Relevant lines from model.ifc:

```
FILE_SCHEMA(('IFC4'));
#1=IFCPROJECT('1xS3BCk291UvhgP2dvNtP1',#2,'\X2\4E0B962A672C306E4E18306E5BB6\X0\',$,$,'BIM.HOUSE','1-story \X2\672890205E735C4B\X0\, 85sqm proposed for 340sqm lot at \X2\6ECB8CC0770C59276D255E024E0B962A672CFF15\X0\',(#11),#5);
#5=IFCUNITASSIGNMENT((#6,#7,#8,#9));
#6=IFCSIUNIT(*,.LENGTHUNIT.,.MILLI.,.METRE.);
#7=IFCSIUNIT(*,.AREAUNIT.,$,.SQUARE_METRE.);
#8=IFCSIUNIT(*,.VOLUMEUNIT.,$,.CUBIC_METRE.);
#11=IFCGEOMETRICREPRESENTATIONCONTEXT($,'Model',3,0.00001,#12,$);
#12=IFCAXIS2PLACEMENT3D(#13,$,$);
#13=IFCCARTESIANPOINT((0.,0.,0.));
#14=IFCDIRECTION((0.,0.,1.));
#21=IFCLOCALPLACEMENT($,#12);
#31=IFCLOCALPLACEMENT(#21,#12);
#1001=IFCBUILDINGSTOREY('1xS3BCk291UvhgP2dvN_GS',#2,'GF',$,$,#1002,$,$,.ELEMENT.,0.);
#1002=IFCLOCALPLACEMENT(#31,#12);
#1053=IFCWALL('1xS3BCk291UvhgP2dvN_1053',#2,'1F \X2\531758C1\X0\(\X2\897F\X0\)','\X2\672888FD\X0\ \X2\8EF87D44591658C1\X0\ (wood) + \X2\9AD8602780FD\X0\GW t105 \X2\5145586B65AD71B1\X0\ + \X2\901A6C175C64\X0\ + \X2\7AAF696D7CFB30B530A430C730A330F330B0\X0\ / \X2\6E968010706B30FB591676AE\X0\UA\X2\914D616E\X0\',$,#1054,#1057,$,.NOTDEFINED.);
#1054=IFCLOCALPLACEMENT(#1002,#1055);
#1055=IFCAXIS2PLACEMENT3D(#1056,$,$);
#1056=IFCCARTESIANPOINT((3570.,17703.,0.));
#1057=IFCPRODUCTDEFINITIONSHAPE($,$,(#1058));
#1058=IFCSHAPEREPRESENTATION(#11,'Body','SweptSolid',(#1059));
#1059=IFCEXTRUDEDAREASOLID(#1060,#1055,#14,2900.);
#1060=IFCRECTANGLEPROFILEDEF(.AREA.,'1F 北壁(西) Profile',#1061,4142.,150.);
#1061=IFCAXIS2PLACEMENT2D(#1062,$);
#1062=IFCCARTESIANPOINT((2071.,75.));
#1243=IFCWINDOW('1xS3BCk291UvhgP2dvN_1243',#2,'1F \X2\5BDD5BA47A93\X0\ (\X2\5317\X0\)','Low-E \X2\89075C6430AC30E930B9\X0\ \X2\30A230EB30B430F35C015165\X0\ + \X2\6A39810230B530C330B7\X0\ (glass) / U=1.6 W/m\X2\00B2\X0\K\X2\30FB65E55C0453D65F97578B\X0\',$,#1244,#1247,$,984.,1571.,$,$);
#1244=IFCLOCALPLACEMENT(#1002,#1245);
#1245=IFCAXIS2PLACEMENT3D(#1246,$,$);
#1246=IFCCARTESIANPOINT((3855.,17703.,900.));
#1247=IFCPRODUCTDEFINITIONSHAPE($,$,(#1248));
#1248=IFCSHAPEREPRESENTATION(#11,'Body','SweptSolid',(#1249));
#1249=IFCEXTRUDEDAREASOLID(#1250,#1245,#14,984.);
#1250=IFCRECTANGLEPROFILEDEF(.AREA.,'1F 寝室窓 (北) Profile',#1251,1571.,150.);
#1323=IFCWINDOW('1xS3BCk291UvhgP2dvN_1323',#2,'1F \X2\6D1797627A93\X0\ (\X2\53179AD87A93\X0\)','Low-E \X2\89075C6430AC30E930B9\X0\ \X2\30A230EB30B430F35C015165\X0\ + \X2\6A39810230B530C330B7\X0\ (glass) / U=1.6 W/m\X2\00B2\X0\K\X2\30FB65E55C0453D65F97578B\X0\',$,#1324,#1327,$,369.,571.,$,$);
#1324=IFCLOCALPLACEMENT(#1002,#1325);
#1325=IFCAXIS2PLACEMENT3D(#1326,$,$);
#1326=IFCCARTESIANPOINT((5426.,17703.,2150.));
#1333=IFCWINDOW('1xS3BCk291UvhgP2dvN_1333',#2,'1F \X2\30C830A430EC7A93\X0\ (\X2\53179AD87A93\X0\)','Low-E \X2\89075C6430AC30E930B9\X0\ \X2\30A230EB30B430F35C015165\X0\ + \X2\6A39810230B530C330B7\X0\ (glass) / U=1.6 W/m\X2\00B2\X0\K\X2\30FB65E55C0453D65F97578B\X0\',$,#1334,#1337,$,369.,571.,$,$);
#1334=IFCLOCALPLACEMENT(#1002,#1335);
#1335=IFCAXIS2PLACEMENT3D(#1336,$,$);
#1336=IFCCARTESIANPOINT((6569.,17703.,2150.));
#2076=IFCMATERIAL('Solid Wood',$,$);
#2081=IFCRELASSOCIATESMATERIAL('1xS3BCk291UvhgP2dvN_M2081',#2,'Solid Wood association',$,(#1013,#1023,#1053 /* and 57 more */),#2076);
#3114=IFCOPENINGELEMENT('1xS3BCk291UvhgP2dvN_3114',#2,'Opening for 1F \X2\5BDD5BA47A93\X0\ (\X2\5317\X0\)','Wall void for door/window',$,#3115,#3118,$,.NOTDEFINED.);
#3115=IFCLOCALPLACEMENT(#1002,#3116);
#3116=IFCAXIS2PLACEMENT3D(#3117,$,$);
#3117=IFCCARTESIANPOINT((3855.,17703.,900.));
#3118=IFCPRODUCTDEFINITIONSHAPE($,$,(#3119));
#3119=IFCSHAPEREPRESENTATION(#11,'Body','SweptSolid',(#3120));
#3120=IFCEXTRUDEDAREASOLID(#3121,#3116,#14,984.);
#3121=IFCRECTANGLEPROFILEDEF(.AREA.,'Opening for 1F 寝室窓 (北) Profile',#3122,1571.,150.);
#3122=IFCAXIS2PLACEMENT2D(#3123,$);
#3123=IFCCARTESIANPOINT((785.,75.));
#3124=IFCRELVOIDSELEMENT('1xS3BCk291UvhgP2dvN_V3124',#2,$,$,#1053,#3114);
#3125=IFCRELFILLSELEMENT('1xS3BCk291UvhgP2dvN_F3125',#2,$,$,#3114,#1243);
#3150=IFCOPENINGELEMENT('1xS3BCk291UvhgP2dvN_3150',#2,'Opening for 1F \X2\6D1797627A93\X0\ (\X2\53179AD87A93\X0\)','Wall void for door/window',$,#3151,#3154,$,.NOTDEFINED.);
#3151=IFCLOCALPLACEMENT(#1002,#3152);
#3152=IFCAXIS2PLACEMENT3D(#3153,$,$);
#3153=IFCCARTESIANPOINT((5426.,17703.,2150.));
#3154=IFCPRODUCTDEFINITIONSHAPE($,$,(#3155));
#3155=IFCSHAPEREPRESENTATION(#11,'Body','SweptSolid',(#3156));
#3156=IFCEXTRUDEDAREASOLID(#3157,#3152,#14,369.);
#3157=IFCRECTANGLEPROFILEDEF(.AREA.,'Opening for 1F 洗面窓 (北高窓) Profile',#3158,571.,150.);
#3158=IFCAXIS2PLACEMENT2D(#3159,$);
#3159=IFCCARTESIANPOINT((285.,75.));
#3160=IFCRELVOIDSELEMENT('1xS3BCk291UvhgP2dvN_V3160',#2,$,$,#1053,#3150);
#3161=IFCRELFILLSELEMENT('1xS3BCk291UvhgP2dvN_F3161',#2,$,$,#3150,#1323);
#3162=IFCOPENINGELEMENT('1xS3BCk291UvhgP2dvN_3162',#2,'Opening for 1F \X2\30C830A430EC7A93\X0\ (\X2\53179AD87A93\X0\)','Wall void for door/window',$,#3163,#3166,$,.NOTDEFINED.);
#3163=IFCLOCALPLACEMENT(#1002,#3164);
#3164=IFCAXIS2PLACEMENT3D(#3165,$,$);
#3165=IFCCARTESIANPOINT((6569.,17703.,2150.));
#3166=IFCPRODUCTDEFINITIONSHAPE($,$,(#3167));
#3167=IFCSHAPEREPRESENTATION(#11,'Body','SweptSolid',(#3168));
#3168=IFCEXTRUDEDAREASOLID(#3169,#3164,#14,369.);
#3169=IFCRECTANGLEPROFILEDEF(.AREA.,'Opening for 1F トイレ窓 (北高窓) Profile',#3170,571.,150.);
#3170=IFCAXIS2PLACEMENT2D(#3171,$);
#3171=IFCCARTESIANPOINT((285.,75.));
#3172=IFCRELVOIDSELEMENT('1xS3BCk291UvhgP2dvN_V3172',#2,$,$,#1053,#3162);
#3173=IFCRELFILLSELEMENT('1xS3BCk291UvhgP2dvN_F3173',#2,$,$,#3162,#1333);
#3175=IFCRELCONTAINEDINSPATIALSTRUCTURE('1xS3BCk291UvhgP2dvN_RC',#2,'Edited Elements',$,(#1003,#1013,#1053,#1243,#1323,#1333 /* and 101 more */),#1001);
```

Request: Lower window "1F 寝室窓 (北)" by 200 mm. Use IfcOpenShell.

```python
import numpy as np
import ifcopenshell
import ifcopenshell.api.geometry
import ifcopenshell.util.placement
import ifcopenshell.util.unit

model = ifcopenshell.open("model.ifc")
unit_scale = ifcopenshell.util.unit.calculate_unit_scale(model)

window = model.by_guid("1xS3BCk291UvhgP2dvN_1243")
opening = window.FillsVoids[0].RelatingOpeningElement
dz = -0.2 / unit_scale

shift = np.array([0.0, 0.0, dz])
# The window is not placed relative to its opening, so move both.
for product in (opening, window):
    matrix = ifcopenshell.util.placement.get_local_placement(product.ObjectPlacement)
    matrix[:3, 3] += shift
    ifcopenshell.api.geometry.edit_object_placement(model, product=product, matrix=matrix, is_si=False)

print(f"moved by {dz * unit_scale:+.3f} m")

model.write("model_updated.ifc")
```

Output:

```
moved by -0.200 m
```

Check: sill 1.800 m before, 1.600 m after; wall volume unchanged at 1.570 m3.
